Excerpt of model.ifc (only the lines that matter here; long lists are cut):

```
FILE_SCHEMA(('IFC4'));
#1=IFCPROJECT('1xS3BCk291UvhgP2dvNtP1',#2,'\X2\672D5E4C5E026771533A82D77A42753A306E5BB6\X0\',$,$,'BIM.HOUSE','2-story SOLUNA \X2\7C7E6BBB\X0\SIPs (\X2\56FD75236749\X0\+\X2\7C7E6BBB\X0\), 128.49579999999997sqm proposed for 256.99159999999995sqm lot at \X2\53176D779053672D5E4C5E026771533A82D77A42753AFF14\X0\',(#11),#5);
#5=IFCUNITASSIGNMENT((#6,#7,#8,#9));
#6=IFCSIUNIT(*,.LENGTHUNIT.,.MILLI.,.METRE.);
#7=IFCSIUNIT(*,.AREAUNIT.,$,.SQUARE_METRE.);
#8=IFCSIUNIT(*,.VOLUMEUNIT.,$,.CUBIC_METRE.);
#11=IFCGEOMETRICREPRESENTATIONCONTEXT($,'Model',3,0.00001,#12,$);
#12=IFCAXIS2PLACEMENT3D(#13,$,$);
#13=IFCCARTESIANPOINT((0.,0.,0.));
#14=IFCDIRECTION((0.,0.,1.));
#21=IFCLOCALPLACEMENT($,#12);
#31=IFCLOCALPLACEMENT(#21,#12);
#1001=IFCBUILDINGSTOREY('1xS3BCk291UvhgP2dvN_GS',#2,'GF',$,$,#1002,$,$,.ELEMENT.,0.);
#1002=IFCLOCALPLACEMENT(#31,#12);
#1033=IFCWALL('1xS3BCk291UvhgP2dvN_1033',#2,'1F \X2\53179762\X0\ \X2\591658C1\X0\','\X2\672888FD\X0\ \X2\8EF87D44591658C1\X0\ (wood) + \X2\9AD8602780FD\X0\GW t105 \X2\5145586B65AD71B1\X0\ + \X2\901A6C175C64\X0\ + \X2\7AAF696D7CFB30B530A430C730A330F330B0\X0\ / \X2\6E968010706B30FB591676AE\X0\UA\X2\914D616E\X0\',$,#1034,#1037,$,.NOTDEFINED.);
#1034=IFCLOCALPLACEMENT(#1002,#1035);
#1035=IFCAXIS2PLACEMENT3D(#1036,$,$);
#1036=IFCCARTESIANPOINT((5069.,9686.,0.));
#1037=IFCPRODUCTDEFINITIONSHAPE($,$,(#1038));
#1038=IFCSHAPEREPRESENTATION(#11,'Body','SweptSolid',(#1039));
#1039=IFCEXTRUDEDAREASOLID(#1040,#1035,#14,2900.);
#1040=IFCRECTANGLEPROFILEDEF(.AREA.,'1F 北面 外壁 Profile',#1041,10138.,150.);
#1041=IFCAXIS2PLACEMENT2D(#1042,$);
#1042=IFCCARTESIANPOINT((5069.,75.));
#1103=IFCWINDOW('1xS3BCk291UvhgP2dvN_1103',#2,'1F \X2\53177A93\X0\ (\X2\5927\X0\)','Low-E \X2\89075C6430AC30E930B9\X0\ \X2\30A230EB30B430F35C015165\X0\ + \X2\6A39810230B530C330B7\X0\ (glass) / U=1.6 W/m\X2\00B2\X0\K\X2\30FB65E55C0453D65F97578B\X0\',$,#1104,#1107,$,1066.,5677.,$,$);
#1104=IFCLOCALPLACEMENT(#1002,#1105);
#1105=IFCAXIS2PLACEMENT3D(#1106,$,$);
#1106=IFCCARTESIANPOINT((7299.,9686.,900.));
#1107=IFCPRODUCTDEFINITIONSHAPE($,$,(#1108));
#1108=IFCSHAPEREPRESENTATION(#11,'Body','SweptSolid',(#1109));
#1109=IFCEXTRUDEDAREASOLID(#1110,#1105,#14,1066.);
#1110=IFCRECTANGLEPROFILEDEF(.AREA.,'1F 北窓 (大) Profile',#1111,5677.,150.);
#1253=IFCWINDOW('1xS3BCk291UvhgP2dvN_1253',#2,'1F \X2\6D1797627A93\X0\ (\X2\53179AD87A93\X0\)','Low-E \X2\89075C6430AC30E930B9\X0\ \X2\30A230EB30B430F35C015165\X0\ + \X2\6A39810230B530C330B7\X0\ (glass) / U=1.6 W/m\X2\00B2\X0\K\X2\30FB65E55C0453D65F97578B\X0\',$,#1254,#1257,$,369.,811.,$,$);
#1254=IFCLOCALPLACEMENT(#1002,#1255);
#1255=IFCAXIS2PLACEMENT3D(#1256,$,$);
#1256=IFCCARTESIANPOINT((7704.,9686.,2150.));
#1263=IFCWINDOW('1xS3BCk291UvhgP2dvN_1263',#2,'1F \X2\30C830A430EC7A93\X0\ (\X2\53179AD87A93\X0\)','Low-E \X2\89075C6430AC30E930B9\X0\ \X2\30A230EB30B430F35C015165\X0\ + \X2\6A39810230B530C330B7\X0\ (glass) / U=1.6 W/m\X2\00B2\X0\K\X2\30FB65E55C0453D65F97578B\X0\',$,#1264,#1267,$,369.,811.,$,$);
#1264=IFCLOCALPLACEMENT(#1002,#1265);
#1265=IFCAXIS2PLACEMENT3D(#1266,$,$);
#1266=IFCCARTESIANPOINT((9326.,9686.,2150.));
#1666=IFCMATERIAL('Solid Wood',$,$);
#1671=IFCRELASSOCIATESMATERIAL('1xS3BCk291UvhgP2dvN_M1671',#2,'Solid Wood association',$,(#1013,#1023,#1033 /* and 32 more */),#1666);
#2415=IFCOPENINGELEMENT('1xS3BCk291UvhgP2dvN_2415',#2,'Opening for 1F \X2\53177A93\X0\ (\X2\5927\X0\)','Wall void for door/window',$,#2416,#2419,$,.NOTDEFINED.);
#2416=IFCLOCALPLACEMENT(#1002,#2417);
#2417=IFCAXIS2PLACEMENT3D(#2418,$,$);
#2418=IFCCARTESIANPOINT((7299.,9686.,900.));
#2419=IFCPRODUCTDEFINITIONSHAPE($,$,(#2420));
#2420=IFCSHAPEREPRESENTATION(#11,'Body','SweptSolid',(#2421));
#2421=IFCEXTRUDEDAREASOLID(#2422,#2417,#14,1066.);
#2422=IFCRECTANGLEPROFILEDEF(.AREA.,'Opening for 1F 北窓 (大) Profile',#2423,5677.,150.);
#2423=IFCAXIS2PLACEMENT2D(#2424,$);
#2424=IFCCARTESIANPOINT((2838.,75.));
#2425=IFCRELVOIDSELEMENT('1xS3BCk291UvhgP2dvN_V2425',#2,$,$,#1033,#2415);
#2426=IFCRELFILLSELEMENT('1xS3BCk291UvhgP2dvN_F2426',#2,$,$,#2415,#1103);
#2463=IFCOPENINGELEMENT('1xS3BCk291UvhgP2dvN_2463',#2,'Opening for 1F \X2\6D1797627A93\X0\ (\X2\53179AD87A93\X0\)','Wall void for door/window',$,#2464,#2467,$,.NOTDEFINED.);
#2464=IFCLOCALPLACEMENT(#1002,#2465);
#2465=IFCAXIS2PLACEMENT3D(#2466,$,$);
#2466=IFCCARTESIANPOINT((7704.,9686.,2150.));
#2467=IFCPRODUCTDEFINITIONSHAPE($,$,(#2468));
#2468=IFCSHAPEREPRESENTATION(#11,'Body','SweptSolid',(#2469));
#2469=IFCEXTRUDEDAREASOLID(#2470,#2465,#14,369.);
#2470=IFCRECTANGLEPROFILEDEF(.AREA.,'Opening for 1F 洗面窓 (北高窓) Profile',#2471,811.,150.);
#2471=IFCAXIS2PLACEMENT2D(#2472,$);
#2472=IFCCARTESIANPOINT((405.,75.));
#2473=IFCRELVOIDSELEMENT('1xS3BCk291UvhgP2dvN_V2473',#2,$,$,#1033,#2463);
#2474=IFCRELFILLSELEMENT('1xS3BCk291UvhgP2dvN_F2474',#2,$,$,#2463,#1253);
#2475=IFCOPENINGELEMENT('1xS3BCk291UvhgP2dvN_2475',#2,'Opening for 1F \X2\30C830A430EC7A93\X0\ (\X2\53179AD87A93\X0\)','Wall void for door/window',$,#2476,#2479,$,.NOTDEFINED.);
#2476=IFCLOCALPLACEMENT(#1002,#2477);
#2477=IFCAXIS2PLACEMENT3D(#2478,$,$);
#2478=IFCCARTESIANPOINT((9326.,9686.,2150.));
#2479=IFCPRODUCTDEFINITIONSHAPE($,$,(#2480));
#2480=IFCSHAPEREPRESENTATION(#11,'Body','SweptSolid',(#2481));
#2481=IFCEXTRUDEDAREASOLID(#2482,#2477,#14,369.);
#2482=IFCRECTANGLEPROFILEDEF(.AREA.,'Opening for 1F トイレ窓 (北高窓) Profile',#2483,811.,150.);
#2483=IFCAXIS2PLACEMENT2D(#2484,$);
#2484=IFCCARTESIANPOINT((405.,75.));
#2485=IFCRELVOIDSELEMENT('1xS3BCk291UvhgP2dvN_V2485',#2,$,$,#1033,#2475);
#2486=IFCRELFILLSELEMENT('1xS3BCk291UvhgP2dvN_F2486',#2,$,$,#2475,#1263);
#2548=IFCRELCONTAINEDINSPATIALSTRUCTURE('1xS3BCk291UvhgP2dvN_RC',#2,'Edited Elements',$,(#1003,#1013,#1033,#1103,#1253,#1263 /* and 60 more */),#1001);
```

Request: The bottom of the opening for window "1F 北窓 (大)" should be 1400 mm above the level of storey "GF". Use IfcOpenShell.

```python
import numpy as np
import ifcopenshell
import ifcopenshell.api.geometry
import ifcopenshell.geom
import ifcopenshell.util.element
import ifcopenshell.util.placement
import ifcopenshell.util.shape
import ifcopenshell.util.unit

model = ifcopenshell.open("model.ifc")
unit_scale = ifcopenshell.util.unit.calculate_unit_scale(model)

window = model.by_guid("1xS3BCk291UvhgP2dvN_1103")
opening = window.FillsVoids[0].RelatingOpeningElement
storey = ifcopenshell.util.element.get_container(window, ifc_class="IfcBuildingStorey")
level = ifcopenshell.util.placement.get_local_placement(storey.ObjectPlacement)[2, 3]

# The opening's origin need not be at the sill, so measure its lowest point.
shape = ifcopenshell.geom.create_shape(ifcopenshell.geom.settings(), opening)
bottom = ifcopenshell.util.shape.get_shape_bottom_elevation(shape, shape.geometry) / unit_scale
dz = level + 1400.0 - bottom

shift = np.array([0.0, 0.0, dz])
# The window is not placed relative to its opening, so move both.
for product in (opening, window):
    matrix = ifcopenshell.util.placement.get_local_placement(product.ObjectPlacement)
    matrix[:3, 3] += shift
    ifcopenshell.api.geometry.edit_object_placement(model, product=product, matrix=matrix, is_si=False)

print(f"moved by {dz * unit_scale:+.3f} m")

model.write("model_edited.ifc")
```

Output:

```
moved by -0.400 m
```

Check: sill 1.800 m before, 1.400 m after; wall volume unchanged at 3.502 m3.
